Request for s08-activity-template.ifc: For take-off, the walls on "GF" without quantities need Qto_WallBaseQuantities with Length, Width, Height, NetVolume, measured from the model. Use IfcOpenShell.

First a look at what the model holds.

```python
import ifcopenshell
import ifcopenshell.util.element
import ifcopenshell.util.unit

model = ifcopenshell.open("s08-activity-template.ifc")
print(model.schema)
for unit_type in ("LENGTHUNIT", "AREAUNIT", "VOLUMEUNIT"):
    print(unit_type, ifcopenshell.util.unit.calculate_unit_scale(model, unit_type))
storey = next(s for s in model.by_type("IfcBuildingStorey") if s.Name == "GF")
walls = [e for e in ifcopenshell.util.element.get_decomposition(storey) if e.is_a("IfcWall")]
for e in sorted(walls, key=lambda e: e.id()):
    print(e.id(), e.is_a(), e.Name, list(ifcopenshell.util.element.get_psets(e, qtos_only=True)), sep=" | ")
```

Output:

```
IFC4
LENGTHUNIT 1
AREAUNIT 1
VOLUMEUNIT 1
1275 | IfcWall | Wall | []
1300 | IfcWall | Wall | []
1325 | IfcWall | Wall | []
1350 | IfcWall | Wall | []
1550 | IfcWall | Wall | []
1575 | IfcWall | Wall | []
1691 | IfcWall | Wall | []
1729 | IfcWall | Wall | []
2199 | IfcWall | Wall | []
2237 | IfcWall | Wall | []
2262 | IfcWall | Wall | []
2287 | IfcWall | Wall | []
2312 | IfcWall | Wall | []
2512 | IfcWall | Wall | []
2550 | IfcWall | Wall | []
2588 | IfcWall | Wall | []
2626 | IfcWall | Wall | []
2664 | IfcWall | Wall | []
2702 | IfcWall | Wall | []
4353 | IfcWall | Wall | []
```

```python
import ifcopenshell
import ifcopenshell.api.pset
import ifcopenshell.geom
import ifcopenshell.util.element
import ifcopenshell.util.shape
import ifcopenshell.util.unit

model = ifcopenshell.open("s08-activity-template.ifc")
unit_scale = ifcopenshell.util.unit.calculate_unit_scale(model)
volume_scale = ifcopenshell.util.unit.calculate_unit_scale(model, "VOLUMEUNIT")
settings = ifcopenshell.geom.settings()

storey = next(s for s in model.by_type("IfcBuildingStorey") if s.Name == "GF")
walls = [e for e in ifcopenshell.util.element.get_decomposition(storey) if e.is_a("IfcWall")]

for e in sorted(walls, key=lambda e: e.id()):
    if ifcopenshell.util.element.get_psets(e, qtos_only=True, should_inherit=False):
        continue
    # Geometry comes back in metres, in the element's own axes.
    shape = ifcopenshell.geom.create_shape(settings, e)
    values = {
        "Length": ifcopenshell.util.shape.get_x(shape.geometry) / unit_scale,
        "Width": ifcopenshell.util.shape.get_y(shape.geometry) / unit_scale,
        "Height": ifcopenshell.util.shape.get_z(shape.geometry) / unit_scale,
        "NetVolume": ifcopenshell.util.shape.get_volume(shape.geometry) / volume_scale,
    }
    qto = ifcopenshell.api.pset.add_qto(model, product=e, name="Qto_WallBaseQuantities")
    ifcopenshell.api.pset.edit_qto(model, qto=qto, properties=values)
    print(e.id(), {k: round(v, 3) for k, v in values.items()})

model.write("s08-activity-template_rev.ifc")
```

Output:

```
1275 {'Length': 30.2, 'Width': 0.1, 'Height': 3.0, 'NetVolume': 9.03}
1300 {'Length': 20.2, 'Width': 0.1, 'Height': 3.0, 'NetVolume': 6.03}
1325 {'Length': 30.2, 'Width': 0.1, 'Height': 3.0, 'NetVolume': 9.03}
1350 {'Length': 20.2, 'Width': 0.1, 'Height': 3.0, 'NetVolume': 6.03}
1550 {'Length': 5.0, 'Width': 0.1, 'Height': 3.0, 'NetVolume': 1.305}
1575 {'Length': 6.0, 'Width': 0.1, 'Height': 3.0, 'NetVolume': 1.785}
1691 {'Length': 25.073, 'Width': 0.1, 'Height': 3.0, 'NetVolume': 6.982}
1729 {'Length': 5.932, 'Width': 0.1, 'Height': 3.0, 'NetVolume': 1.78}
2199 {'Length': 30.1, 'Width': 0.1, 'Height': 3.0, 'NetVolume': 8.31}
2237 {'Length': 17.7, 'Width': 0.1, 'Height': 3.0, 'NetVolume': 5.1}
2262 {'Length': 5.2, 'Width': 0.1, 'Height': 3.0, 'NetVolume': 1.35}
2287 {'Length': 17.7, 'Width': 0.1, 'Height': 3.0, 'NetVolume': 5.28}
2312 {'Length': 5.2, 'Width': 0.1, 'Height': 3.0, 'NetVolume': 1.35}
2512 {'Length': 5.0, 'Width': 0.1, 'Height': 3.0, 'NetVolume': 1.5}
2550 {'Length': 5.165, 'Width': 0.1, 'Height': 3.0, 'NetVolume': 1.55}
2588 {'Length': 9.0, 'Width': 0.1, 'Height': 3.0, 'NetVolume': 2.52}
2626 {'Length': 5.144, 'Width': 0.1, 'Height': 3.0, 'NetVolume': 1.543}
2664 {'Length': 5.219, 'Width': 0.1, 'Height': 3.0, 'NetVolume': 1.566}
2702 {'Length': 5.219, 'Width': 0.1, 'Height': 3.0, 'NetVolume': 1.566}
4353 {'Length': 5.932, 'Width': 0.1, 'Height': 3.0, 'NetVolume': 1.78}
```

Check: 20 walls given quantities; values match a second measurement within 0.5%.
